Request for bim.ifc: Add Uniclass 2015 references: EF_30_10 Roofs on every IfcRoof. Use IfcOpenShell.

First a look at what the model holds.

```python
import ifcopenshell

model = ifcopenshell.open("bim.ifc")
print(model.schema)
print("classifications:", [c.Name for c in model.by_type("IfcClassification")])
for ifc_class in ("IfcDoor", "IfcRoof", "IfcStair", "IfcWall", "IfcWindow"):
    print(ifc_class, len(model.by_type(ifc_class)))
```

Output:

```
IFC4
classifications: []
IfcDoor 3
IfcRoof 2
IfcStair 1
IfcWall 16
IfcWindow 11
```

```python
import ifcopenshell
import ifcopenshell.api.classification

model = ifcopenshell.open("bim.ifc")

system = ifcopenshell.api.classification.add_classification(model, classification="Uniclass 2015")

codes = {
    "IfcRoof": ("EF_30_10", "Roofs"),
}
for ifc_class, (code, name) in codes.items():
    products = model.by_type(ifc_class)
    ifcopenshell.api.classification.add_reference(
        model, products=products, classification=system, identification=code, name=name
    )
    print(code, len(products))

model.write("bim_updated.ifc")
```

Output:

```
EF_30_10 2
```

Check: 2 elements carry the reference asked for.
